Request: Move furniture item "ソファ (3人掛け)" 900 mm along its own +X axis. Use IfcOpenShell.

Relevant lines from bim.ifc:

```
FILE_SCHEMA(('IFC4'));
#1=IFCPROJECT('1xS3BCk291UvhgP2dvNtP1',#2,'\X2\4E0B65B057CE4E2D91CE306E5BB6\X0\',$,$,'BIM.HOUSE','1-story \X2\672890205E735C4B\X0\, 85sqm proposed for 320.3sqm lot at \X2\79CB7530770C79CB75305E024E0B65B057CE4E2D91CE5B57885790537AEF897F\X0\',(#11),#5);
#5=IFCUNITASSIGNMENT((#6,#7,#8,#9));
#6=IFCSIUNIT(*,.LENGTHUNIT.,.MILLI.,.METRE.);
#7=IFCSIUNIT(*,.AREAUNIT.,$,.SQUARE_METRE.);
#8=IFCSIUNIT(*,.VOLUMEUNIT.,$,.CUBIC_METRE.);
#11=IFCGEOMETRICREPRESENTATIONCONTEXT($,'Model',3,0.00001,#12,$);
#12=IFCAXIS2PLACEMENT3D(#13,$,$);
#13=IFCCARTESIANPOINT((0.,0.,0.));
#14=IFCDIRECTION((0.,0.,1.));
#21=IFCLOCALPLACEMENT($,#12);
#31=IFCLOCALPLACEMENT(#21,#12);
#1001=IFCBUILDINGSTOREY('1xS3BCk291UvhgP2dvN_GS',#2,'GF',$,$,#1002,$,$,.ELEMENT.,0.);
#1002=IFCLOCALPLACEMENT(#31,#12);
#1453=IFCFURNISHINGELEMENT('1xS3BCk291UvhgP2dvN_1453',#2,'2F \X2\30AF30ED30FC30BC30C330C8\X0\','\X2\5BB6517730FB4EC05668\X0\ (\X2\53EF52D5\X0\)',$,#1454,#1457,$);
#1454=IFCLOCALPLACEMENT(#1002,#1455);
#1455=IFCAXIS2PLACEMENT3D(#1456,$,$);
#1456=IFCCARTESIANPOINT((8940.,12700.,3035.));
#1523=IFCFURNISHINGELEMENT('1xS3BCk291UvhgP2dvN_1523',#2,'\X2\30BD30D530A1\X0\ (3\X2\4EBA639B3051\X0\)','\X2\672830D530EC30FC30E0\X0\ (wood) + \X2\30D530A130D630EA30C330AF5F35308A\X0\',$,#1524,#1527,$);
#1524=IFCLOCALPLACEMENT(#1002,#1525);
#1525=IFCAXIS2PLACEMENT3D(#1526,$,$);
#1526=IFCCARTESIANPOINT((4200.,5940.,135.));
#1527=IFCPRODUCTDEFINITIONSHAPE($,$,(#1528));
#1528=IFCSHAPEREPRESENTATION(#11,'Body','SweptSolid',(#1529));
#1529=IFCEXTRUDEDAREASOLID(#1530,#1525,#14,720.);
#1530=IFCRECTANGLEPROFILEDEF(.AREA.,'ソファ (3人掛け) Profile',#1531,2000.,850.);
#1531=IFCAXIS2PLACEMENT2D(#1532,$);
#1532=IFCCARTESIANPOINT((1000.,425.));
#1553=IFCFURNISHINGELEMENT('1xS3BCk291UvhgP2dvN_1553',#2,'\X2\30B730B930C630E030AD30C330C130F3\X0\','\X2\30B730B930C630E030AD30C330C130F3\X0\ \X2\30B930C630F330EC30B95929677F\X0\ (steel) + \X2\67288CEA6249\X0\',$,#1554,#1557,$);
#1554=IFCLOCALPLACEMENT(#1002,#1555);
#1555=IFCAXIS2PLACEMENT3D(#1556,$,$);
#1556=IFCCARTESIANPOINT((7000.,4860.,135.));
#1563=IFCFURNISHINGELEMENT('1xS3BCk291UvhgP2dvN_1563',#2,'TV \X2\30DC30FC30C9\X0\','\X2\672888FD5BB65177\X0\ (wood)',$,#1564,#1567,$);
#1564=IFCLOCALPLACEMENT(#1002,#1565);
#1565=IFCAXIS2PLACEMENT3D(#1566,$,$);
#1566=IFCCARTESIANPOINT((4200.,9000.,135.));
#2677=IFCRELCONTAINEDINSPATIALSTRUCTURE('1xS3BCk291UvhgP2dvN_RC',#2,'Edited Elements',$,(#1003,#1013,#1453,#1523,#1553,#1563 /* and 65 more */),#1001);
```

```python
import ifcopenshell
import ifcopenshell.api.geometry
import ifcopenshell.util.placement
import ifcopenshell.util.unit

model = ifcopenshell.open("bim.ifc")
unit_scale = ifcopenshell.util.unit.calculate_unit_scale(model)

item = model.by_guid("1xS3BCk291UvhgP2dvN_1523")
matrix = ifcopenshell.util.placement.get_local_placement(item.ObjectPlacement)
matrix[:3, 3] += matrix[:3, 0] * 0.9 / unit_scale
ifcopenshell.api.geometry.edit_object_placement(model, product=item, matrix=matrix, is_si=False)

print(ifcopenshell.util.placement.get_local_placement(item.ObjectPlacement).round(3) + 0.0)

model.write("bim-out.ifc")
```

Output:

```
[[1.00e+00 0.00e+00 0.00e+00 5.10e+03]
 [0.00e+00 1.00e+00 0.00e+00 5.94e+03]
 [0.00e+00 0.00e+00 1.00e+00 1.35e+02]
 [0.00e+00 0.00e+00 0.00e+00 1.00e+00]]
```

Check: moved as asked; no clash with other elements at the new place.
